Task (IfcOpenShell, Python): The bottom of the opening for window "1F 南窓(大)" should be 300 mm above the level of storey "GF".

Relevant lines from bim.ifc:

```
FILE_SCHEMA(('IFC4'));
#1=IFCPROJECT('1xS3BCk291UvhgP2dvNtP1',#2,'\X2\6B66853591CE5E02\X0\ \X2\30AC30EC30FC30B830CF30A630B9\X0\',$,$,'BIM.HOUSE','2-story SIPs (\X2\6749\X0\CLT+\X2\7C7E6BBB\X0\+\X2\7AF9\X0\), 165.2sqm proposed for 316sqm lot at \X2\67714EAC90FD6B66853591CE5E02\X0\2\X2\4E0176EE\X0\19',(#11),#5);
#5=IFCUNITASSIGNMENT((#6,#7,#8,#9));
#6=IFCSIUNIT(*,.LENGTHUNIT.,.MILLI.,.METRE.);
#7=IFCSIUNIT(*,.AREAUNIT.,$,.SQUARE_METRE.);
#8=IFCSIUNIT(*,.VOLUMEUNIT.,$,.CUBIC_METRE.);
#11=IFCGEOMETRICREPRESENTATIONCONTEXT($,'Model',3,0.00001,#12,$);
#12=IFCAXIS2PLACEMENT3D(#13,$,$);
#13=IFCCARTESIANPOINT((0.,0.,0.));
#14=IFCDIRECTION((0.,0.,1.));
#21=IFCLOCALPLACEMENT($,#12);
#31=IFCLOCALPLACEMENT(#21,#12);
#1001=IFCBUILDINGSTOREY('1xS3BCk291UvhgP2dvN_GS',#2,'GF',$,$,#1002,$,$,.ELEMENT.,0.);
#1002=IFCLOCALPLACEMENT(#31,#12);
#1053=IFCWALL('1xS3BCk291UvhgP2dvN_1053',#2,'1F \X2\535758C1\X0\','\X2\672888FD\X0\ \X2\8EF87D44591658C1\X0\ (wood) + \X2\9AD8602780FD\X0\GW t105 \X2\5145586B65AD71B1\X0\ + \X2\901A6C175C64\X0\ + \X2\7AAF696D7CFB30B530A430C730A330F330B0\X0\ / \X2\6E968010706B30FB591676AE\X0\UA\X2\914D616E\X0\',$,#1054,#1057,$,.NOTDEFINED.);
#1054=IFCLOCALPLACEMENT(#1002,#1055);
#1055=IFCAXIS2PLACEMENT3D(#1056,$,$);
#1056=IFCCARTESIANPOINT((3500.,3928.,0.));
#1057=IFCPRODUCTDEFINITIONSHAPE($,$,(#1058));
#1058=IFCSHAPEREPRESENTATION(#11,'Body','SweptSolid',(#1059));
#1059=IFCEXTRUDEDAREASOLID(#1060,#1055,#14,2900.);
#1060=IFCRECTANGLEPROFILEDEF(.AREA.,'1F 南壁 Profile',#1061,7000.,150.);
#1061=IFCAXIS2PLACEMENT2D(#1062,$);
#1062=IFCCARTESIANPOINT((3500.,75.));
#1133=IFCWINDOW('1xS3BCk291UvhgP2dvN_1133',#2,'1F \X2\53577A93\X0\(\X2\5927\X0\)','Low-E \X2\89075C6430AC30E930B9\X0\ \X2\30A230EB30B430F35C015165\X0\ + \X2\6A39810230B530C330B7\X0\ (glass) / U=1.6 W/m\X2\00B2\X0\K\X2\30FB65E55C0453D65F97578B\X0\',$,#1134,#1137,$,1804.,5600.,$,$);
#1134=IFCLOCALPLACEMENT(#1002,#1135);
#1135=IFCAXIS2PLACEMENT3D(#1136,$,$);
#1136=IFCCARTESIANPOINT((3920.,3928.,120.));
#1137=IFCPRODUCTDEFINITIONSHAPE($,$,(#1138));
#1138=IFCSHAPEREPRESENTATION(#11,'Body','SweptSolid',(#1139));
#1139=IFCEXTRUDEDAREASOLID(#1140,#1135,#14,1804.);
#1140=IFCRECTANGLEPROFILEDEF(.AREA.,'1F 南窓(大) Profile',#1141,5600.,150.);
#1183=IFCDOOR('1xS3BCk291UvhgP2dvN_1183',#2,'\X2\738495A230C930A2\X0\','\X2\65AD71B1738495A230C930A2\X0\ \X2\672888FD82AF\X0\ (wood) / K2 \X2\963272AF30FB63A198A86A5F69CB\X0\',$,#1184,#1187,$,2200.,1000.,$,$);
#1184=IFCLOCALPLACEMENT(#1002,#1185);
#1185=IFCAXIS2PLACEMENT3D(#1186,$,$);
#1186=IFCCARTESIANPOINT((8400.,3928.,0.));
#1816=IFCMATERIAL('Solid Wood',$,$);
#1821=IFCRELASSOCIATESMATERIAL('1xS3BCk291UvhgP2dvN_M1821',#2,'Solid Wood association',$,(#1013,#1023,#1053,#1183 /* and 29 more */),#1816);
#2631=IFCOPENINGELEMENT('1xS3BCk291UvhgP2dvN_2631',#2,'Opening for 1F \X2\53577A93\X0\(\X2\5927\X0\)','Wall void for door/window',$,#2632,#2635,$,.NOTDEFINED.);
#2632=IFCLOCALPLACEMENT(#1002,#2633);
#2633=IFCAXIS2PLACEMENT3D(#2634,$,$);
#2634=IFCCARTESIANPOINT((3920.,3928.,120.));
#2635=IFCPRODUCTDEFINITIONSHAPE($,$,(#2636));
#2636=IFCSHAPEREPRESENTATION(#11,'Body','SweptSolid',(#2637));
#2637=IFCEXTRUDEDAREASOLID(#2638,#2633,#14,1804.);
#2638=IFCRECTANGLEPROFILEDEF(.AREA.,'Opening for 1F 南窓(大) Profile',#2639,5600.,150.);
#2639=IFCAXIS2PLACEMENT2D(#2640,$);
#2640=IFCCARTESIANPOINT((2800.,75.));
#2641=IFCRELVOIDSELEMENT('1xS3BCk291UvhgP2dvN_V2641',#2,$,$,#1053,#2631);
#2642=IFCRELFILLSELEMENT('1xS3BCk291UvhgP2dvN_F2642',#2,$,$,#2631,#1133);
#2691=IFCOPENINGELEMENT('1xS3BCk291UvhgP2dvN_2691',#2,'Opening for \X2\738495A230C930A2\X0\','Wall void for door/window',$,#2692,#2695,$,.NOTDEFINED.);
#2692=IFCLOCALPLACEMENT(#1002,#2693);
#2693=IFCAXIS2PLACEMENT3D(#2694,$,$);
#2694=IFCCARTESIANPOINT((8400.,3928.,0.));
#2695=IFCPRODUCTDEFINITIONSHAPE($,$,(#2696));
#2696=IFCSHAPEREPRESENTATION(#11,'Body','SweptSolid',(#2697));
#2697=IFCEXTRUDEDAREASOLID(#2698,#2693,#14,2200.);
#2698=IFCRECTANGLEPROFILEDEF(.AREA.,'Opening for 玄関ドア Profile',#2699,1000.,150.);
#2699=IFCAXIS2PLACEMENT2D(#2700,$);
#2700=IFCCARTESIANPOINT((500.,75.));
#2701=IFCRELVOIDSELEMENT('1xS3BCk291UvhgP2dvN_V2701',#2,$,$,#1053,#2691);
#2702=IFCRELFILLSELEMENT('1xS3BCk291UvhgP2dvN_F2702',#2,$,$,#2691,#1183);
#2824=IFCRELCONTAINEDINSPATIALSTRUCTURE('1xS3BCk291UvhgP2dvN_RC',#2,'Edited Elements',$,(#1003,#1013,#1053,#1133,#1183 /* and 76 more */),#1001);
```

```python
import numpy as np
import ifcopenshell
import ifcopenshell.api.geometry
import ifcopenshell.geom
import ifcopenshell.util.element
import ifcopenshell.util.placement
import ifcopenshell.util.shape
import ifcopenshell.util.unit

model = ifcopenshell.open("bim.ifc")
unit_scale = ifcopenshell.util.unit.calculate_unit_scale(model)

window = model.by_id(1133)
opening = window.FillsVoids[0].RelatingOpeningElement
storey = ifcopenshell.util.element.get_container(window, ifc_class="IfcBuildingStorey")
level = ifcopenshell.util.placement.get_local_placement(storey.ObjectPlacement)[2, 3]

# The opening's origin need not be at the sill, so measure its lowest point.
shape = ifcopenshell.geom.create_shape(ifcopenshell.geom.settings(), opening)
bottom = ifcopenshell.util.shape.get_shape_bottom_elevation(shape, shape.geometry) / unit_scale
dz = level + 0.3 / unit_scale - bottom

shift = np.array([0.0, 0.0, dz])
# The window is not placed relative to its opening, so move both.
for product in (opening, window):
    matrix = ifcopenshell.util.placement.get_local_placement(product.ObjectPlacement)
    matrix[:3, 3] += shift
    ifcopenshell.api.geometry.edit_object_placement(model, product=product, matrix=matrix, is_si=False)

print(f"moved by {dz * unit_scale:+.3f} m")

model.write("bim_rev.ifc")
```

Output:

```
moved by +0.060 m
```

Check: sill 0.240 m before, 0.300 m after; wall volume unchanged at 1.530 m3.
